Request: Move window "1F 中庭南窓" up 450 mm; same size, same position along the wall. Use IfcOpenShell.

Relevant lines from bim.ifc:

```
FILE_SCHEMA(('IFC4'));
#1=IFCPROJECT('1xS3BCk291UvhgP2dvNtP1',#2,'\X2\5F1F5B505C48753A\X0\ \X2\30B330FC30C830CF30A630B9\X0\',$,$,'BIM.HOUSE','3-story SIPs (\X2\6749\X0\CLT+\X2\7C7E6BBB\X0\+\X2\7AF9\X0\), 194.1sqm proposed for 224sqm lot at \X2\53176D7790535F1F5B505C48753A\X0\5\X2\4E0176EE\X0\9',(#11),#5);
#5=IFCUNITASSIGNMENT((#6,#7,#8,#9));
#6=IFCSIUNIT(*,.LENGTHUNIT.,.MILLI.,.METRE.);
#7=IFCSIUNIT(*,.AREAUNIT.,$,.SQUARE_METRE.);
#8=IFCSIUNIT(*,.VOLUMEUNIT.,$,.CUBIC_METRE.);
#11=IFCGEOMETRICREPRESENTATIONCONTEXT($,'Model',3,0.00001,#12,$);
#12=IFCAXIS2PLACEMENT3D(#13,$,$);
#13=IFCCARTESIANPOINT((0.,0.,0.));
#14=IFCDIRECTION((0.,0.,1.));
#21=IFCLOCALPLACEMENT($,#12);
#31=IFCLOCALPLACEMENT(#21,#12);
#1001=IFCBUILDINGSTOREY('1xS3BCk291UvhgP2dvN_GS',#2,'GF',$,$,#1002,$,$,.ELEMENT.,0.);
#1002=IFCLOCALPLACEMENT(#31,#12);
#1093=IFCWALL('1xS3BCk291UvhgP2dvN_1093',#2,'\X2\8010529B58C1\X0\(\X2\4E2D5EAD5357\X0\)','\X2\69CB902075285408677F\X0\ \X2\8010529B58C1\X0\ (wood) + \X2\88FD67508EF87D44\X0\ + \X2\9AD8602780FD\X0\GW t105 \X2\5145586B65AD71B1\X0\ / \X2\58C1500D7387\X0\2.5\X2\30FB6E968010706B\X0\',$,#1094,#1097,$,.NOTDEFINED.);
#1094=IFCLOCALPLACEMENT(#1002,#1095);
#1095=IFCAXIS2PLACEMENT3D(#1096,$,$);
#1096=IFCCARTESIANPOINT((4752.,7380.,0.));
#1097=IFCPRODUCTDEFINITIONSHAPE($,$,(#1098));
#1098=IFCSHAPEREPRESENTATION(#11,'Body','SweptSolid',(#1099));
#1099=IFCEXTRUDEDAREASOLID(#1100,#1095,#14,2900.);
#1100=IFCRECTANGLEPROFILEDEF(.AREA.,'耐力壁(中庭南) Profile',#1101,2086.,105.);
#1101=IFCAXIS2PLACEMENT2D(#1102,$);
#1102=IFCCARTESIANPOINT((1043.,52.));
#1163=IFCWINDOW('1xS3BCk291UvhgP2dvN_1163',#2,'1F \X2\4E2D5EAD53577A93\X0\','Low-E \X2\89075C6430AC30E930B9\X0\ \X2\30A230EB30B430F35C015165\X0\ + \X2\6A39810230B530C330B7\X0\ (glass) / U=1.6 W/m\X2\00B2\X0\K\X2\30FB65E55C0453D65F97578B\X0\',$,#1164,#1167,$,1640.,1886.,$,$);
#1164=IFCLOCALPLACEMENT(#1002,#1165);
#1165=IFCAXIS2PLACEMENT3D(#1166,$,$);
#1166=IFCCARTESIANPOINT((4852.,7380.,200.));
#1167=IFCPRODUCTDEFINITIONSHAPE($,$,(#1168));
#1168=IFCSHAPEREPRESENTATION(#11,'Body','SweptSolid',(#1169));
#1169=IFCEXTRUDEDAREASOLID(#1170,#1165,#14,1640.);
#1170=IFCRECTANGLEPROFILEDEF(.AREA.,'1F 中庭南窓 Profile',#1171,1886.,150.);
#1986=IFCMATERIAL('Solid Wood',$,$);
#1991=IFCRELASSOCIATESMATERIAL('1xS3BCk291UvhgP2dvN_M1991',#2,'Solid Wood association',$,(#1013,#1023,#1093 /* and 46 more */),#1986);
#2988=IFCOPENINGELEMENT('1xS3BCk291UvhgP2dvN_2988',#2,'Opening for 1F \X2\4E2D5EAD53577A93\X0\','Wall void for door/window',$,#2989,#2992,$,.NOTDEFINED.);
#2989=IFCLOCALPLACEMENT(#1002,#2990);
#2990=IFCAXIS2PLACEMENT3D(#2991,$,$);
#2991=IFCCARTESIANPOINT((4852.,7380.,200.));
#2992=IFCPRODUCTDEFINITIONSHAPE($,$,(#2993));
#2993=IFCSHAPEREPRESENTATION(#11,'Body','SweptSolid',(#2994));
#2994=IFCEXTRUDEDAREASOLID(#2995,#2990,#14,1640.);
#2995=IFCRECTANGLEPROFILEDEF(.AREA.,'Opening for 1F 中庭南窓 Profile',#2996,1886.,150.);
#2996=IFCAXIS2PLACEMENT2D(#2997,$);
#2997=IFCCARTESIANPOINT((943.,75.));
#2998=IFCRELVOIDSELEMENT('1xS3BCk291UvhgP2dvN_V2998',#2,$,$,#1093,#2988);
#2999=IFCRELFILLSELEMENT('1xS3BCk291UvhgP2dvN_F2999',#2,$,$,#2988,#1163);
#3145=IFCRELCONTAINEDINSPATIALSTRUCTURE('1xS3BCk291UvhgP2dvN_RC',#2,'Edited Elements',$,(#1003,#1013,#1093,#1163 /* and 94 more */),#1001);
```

```python
import numpy as np
import ifcopenshell
import ifcopenshell.api.geometry
import ifcopenshell.util.placement
import ifcopenshell.util.unit

model = ifcopenshell.open("bim.ifc")
unit_scale = ifcopenshell.util.unit.calculate_unit_scale(model)

window = model.by_guid("1xS3BCk291UvhgP2dvN_1163")
opening = window.FillsVoids[0].RelatingOpeningElement
dz = 450.0

shift = np.array([0.0, 0.0, dz])
# The window is not placed relative to its opening, so move both.
for product in (opening, window):
    matrix = ifcopenshell.util.placement.get_local_placement(product.ObjectPlacement)
    matrix[:3, 3] += shift
    ifcopenshell.api.geometry.edit_object_placement(model, product=product, matrix=matrix, is_si=False)

print(f"moved by {dz * unit_scale:+.3f} m")

model.write("bim_updated.ifc")
```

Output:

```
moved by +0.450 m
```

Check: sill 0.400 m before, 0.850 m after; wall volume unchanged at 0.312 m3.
